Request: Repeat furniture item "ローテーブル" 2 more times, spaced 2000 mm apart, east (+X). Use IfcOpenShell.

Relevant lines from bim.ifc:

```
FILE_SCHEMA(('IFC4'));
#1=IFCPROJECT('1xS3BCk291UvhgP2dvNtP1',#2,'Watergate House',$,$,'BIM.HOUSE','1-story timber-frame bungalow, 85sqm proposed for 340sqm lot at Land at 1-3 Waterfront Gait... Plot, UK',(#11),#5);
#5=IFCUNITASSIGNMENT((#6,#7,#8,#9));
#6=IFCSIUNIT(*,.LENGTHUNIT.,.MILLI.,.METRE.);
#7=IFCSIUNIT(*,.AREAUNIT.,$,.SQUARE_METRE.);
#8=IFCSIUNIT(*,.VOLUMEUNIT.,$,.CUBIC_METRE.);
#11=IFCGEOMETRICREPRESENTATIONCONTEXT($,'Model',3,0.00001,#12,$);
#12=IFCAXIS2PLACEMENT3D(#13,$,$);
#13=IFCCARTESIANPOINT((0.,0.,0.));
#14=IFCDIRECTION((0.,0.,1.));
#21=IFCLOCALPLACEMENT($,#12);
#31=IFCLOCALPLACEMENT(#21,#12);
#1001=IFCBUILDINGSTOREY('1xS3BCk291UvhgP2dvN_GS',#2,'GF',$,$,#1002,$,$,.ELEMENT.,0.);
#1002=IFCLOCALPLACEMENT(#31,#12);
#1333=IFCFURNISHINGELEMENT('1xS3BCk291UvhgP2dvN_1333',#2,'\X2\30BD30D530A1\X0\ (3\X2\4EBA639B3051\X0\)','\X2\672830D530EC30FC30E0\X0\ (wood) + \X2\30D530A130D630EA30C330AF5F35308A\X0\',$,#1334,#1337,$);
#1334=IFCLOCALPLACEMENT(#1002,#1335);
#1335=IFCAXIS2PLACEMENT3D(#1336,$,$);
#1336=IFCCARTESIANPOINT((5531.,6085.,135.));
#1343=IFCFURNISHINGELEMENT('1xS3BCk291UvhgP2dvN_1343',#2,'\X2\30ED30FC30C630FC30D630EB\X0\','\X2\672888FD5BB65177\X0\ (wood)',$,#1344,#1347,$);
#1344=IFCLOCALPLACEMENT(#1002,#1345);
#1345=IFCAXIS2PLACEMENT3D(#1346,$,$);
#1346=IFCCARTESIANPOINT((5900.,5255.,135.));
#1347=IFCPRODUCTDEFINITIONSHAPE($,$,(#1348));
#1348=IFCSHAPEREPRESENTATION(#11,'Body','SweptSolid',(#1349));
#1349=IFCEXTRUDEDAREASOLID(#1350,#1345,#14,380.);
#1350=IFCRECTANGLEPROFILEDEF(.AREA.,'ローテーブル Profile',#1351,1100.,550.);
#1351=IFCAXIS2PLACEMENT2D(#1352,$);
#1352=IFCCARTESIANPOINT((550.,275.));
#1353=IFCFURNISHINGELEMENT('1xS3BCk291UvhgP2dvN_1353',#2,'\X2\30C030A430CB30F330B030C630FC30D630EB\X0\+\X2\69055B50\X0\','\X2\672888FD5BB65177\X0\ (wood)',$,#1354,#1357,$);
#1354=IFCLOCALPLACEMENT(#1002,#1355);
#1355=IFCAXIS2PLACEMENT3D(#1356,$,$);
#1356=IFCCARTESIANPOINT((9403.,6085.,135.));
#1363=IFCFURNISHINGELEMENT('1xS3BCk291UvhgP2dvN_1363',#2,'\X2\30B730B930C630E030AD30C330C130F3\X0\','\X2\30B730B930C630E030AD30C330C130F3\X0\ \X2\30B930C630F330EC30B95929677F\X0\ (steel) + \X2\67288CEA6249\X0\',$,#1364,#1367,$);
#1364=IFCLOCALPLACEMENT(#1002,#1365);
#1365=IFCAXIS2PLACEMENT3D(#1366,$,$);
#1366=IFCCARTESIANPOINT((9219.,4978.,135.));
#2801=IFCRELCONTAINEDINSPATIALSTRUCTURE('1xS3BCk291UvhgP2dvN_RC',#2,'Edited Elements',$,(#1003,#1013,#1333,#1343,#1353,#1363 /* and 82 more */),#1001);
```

```python
import numpy as np
import ifcopenshell
import ifcopenshell.api.geometry
import ifcopenshell.api.root
import ifcopenshell.util.element
import ifcopenshell.util.placement

model = ifcopenshell.open("bim.ifc")


def reuse_history(source, copy):
    """copy_class also copies each property set's owner history, people and application; keep the originals."""
    for rel in copy.IsDefinedBy:
        if rel.is_a("IfcRelDefinesByProperties") and (history := rel.RelatingPropertyDefinition.OwnerHistory):
            rel.RelatingPropertyDefinition.OwnerHistory = source.OwnerHistory
            ifcopenshell.util.element.remove_deep2(model, history)


source = model.by_guid("1xS3BCk291UvhgP2dvN_1343")
base = ifcopenshell.util.placement.get_local_placement(source.ObjectPlacement)
step = np.array([1.0, 0.0, 0.0]) * 2000.0

for i in range(1, 3):
    copy = ifcopenshell.api.root.copy_class(model, product=source)
    copy.Representation = ifcopenshell.util.element.copy_deep(
        model, source.Representation, exclude=["IfcGeometricRepresentationContext", "IfcRepresentationMap"]
    )
    reuse_history(source, copy)
    matrix = base.copy()
    matrix[:3, 3] += i * step
    print("added at", matrix[:3, 3].round(3) + 0.0)
    ifcopenshell.api.geometry.edit_object_placement(model, product=copy, matrix=matrix, is_si=False)

model.write("bim_rev.ifc")
```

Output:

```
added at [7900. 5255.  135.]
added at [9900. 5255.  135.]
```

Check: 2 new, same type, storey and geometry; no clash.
